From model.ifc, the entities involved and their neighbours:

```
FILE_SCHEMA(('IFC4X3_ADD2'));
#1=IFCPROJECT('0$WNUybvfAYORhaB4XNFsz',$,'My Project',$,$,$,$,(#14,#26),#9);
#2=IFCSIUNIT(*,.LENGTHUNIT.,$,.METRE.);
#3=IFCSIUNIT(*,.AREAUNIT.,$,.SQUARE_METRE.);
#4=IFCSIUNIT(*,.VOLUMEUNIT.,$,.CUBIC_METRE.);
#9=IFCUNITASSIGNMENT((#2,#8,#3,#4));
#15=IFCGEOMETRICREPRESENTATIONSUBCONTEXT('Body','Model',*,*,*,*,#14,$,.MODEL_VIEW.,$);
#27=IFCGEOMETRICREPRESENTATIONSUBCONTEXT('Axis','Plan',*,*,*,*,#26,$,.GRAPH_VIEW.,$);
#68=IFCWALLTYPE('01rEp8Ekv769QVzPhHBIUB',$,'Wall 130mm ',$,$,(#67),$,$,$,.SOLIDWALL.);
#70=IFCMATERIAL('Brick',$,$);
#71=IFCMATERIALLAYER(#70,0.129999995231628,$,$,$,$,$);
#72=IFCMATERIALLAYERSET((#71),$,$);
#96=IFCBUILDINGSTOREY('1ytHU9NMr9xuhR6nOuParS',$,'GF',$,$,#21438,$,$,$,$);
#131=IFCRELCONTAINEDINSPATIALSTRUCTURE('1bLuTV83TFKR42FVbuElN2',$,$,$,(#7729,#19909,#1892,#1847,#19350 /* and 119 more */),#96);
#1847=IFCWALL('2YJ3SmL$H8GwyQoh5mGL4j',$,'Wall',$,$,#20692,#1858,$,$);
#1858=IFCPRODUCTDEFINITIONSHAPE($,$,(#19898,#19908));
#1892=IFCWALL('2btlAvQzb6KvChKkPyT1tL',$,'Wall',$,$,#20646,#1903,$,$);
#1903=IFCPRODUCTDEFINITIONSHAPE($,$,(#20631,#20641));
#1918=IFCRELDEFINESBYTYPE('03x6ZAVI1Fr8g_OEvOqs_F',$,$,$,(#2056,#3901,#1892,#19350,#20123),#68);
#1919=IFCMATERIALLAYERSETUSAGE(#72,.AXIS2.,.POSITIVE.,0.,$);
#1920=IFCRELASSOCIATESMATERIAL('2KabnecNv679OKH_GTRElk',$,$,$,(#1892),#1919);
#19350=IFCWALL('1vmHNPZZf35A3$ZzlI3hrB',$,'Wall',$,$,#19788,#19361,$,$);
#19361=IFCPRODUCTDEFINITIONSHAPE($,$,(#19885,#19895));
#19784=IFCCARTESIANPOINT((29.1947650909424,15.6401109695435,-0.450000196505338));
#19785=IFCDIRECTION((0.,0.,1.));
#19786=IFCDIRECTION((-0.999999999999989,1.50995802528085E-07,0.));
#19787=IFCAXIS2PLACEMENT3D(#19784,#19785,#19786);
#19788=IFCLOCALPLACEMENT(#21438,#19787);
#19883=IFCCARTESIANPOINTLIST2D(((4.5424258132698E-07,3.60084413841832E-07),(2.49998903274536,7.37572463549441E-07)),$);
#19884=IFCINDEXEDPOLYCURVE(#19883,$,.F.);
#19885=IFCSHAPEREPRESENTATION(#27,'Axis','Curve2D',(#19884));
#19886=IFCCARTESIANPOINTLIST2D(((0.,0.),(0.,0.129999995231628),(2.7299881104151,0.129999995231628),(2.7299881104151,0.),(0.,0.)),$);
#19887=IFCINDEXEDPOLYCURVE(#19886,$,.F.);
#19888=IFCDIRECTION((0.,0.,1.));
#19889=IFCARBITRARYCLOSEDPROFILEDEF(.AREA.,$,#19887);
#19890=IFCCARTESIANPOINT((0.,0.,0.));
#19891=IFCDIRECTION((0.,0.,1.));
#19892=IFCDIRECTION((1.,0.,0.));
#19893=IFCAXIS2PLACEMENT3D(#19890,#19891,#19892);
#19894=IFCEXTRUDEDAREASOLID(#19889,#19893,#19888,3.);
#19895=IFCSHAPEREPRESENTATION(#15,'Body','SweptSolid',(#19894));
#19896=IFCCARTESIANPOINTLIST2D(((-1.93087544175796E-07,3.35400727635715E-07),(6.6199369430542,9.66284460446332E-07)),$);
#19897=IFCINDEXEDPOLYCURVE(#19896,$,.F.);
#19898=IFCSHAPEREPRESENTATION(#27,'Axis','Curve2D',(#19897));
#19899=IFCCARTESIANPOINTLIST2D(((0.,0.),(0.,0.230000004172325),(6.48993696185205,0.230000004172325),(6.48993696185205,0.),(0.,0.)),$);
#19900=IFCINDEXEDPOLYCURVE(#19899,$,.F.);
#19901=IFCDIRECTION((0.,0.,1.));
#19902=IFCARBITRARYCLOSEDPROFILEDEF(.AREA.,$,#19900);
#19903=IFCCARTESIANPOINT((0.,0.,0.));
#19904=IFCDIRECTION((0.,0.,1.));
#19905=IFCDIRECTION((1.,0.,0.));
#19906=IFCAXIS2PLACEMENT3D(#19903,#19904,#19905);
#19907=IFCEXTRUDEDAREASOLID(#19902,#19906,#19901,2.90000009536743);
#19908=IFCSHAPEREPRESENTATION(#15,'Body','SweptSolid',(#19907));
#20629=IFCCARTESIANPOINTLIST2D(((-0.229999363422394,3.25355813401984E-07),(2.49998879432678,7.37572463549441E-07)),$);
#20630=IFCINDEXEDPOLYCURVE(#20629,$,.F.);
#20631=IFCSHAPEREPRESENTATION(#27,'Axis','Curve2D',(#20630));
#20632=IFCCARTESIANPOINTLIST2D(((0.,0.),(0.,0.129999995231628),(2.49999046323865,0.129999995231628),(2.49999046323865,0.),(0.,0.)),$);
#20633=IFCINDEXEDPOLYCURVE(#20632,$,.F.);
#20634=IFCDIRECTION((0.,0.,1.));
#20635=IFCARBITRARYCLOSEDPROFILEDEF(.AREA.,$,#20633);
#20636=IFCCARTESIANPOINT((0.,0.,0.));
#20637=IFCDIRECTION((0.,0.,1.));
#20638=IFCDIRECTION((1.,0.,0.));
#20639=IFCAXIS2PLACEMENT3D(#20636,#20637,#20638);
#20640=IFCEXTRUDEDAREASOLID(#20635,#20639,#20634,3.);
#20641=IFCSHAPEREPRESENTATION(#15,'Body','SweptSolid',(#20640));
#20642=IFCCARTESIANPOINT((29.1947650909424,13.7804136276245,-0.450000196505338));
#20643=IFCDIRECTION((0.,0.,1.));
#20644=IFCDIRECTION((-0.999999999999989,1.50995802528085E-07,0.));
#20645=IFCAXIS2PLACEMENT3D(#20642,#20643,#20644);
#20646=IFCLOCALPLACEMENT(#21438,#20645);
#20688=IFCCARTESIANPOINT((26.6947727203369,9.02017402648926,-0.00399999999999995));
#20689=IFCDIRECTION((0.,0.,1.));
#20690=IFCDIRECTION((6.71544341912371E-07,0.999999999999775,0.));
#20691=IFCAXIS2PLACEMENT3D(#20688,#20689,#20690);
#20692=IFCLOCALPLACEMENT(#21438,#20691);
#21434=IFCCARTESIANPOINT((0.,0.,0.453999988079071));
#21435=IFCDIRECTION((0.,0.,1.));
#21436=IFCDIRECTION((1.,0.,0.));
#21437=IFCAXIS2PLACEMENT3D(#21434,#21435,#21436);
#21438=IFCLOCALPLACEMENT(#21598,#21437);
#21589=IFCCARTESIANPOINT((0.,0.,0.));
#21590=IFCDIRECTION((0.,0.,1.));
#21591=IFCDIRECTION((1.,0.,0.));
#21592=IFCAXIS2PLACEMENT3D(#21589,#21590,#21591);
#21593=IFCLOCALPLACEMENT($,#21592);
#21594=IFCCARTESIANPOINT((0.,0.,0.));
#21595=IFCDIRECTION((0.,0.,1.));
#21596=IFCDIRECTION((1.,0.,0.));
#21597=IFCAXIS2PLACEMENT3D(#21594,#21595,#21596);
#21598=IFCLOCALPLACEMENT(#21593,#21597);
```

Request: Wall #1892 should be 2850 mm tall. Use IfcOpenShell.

```python
import ifcopenshell
import ifcopenshell.geom
import ifcopenshell.util.representation
import ifcopenshell.util.shape
import ifcopenshell.util.unit

model = ifcopenshell.open("model.ifc")
unit_scale = ifcopenshell.util.unit.calculate_unit_scale(model)
settings = ifcopenshell.geom.settings()


def volume(element):
    """Net volume in cubic metres, openings subtracted."""
    shape = ifcopenshell.geom.create_shape(settings, element)
    return ifcopenshell.util.shape.get_volume(shape.geometry)


wall = model.by_id(1892)
before = volume(wall)

body = ifcopenshell.util.representation.get_representation(wall, "Model", "Body")
solid = body.Items[0]
old_height = solid.Depth
solid.Depth = 2.85 / unit_scale
after = volume(wall)

print(f"height {old_height:g} -> {solid.Depth:g}, volume {before:.3f} -> {after:.3f} m3")

model.write("model_updated.ifc")
```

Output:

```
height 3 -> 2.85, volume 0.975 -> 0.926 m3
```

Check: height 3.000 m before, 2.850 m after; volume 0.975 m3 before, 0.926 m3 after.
